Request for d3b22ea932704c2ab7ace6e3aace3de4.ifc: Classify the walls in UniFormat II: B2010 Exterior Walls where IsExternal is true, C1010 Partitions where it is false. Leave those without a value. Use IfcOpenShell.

First a look at what the model holds.

```python
import ifcopenshell
import ifcopenshell.util.element

model = ifcopenshell.open("d3b22ea932704c2ab7ace6e3aace3de4.ifc")
print(model.schema)
print("classifications:", [c.Name for c in model.by_type("IfcClassification")])
values = [ifcopenshell.util.element.get_pset(e, "Pset_WallCommon", "IsExternal") for e in model.by_type("IfcWall")]
for value in (True, False, None):
    print("IsExternal", value, values.count(value))
```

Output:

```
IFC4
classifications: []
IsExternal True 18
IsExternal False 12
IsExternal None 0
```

```python
import ifcopenshell
import ifcopenshell.api.classification
import ifcopenshell.util.element

model = ifcopenshell.open("d3b22ea932704c2ab7ace6e3aace3de4.ifc")

system = ifcopenshell.api.classification.add_classification(model, classification="UniFormat II")

walls = model.by_type("IfcWall")
external = {e: ifcopenshell.util.element.get_pset(e, "Pset_WallCommon", "IsExternal") for e in walls}
for flag, code, name in ((True, "B2010", "Exterior Walls"), (False, "C1010", "Partitions")):
    products = [e for e in walls if external[e] is flag]
    ifcopenshell.api.classification.add_reference(
        model, products=products, classification=system, identification=code, name=name
    )
    print(code, len(products))

model.write("d3b22ea932704c2ab7ace6e3aace3de4_rev.ifc")
```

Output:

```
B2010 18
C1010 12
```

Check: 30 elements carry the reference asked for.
